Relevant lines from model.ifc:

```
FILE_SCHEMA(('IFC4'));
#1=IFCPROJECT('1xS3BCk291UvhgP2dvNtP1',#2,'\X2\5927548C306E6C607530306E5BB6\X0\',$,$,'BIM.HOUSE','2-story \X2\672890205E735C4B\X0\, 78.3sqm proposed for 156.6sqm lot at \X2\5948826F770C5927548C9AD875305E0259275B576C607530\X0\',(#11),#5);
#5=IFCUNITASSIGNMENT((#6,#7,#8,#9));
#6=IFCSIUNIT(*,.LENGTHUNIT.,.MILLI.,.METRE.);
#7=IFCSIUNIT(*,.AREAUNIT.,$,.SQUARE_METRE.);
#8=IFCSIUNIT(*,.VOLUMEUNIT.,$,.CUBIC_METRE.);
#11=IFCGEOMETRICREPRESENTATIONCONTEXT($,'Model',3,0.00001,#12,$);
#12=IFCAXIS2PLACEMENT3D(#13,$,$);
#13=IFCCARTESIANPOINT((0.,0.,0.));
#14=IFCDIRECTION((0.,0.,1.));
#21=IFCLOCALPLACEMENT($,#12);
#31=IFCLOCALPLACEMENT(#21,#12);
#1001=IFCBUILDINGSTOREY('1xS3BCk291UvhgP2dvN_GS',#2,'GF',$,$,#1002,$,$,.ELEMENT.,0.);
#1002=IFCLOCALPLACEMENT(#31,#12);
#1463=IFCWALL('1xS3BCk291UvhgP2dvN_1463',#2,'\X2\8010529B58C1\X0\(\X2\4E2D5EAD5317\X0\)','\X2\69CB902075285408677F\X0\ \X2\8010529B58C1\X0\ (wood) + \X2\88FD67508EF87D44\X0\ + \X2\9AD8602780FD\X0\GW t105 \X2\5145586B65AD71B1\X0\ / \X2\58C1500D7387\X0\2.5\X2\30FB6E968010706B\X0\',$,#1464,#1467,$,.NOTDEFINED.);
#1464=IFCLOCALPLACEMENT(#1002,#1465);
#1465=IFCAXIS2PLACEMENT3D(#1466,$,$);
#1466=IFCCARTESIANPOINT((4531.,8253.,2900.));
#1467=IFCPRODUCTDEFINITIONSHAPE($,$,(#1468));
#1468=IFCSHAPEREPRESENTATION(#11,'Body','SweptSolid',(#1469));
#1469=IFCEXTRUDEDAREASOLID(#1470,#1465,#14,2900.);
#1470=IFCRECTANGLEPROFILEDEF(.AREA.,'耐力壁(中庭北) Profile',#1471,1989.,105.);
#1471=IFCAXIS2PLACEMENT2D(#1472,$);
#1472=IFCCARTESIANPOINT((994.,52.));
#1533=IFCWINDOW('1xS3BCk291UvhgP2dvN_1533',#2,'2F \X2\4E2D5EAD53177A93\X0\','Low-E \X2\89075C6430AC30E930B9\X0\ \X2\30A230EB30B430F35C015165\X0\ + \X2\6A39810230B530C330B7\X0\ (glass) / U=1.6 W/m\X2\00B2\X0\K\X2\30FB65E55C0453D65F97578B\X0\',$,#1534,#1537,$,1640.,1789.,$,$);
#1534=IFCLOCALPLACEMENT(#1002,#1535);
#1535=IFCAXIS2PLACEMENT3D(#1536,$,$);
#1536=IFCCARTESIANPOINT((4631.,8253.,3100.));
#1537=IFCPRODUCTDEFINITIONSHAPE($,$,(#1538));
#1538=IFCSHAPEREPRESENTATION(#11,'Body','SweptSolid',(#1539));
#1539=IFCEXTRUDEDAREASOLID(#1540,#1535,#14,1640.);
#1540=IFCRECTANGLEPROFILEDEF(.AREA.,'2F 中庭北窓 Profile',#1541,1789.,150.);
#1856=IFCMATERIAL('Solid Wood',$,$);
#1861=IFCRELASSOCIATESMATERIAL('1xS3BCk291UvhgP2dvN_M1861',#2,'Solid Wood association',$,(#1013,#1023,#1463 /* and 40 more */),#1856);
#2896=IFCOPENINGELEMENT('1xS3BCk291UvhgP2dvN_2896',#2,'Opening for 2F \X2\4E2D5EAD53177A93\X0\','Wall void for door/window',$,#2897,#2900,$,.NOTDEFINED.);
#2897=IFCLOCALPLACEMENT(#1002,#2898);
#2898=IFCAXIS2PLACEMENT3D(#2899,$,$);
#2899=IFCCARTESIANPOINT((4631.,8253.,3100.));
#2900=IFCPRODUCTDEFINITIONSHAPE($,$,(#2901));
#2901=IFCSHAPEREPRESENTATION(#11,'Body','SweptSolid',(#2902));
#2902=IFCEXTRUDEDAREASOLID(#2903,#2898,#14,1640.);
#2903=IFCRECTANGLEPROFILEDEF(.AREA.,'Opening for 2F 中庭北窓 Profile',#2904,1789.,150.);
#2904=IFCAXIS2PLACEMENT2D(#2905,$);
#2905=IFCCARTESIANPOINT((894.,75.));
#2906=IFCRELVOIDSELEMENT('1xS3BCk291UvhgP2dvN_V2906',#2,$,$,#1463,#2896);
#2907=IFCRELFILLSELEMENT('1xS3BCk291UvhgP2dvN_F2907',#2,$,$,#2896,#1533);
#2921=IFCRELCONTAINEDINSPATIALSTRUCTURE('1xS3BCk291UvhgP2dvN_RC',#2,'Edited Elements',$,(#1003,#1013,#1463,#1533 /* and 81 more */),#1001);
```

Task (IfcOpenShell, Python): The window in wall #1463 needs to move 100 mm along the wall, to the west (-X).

```python
import ifcopenshell
import ifcopenshell.api.geometry
import ifcopenshell.util.placement

model = ifcopenshell.open("model.ifc")

window = model.by_guid("1xS3BCk291UvhgP2dvN_1533")
opening = window.FillsVoids[0].RelatingOpeningElement
wall = opening.VoidsElements[0].RelatingBuildingElement

wall_matrix = ifcopenshell.util.placement.get_local_placement(wall.ObjectPlacement)
shift = wall_matrix[:3, 0] * -100.0
before = ifcopenshell.util.placement.get_local_placement(window.ObjectPlacement)[:3, 3].copy()

# The window is not placed relative to its opening, so move both.
for product in (opening, window):
    matrix = ifcopenshell.util.placement.get_local_placement(product.ObjectPlacement)
    matrix[:3, 3] += shift
    ifcopenshell.api.geometry.edit_object_placement(model, product=product, matrix=matrix, is_si=False)

after = ifcopenshell.util.placement.get_local_placement(window.ObjectPlacement)[:3, 3]
print("window moved by", (after - before).round(3) + 0.0)

model.write("model_edited.ifc")
```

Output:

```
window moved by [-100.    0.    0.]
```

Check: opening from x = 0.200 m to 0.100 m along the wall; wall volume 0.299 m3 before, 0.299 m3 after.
